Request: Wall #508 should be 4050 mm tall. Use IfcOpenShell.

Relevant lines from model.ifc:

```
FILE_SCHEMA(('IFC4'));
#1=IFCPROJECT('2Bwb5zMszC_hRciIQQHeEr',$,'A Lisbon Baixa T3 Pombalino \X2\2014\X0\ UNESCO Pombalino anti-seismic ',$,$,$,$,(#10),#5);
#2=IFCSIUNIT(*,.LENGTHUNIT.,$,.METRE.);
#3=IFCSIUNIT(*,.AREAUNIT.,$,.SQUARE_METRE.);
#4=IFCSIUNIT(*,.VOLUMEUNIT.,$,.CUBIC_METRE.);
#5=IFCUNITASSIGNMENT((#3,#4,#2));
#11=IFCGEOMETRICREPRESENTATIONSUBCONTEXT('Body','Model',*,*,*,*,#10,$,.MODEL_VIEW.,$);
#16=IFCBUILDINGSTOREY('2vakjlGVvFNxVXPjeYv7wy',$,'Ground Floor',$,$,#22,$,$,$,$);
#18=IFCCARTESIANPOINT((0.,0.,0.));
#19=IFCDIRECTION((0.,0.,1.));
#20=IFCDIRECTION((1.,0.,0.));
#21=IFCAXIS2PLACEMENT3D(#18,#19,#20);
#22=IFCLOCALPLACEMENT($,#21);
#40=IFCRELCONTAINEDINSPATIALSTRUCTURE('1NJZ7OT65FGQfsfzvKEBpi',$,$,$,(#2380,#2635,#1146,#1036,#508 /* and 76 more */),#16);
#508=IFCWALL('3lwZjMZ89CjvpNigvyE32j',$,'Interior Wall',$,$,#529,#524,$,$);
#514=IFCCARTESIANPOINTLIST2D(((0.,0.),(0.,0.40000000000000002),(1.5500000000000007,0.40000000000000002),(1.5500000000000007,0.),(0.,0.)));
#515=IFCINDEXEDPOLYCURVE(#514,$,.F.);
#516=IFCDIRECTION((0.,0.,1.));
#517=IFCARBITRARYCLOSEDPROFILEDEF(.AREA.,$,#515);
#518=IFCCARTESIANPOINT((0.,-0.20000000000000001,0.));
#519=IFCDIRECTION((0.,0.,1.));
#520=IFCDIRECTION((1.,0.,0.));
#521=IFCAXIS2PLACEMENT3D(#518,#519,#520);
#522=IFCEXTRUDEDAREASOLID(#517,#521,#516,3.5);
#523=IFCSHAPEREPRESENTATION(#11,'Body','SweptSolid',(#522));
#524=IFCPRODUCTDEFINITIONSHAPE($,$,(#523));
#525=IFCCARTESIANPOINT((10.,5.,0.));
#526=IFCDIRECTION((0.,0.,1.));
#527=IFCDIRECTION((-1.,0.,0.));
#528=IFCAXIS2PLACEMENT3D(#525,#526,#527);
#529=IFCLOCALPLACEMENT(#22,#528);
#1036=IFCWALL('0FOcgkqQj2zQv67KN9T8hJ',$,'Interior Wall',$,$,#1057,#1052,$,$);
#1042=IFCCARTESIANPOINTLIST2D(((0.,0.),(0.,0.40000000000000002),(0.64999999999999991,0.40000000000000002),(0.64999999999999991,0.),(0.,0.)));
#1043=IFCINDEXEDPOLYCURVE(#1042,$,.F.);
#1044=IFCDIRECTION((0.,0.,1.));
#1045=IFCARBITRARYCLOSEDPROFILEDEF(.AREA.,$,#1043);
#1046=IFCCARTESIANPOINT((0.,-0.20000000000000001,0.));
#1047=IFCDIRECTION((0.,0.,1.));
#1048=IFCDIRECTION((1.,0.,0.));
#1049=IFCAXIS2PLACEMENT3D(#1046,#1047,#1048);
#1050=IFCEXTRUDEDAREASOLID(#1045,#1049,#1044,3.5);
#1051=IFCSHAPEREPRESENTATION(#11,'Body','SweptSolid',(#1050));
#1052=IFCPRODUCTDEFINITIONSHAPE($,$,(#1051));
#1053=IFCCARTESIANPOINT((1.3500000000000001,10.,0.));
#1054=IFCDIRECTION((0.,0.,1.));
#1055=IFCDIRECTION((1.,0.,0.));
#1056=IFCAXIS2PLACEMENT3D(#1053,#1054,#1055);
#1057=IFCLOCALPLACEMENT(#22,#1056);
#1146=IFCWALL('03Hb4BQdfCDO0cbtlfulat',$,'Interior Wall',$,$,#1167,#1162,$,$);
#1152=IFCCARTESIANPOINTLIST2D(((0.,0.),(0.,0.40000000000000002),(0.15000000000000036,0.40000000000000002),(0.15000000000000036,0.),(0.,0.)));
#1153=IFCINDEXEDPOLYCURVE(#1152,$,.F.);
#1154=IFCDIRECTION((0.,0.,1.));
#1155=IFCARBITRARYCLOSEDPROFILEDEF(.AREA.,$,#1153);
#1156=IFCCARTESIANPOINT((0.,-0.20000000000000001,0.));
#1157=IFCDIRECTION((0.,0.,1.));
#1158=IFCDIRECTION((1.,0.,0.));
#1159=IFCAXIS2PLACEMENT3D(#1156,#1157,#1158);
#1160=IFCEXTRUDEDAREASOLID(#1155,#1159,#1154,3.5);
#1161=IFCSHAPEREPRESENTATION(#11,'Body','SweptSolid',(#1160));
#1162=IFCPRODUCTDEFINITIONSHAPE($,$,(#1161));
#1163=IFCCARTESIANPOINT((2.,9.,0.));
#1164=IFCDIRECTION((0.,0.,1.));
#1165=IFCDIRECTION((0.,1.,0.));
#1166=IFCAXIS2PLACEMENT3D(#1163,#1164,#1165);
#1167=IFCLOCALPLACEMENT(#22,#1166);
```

```python
import ifcopenshell
import ifcopenshell.geom
import ifcopenshell.util.representation
import ifcopenshell.util.shape
import ifcopenshell.util.unit

model = ifcopenshell.open("model.ifc")
unit_scale = ifcopenshell.util.unit.calculate_unit_scale(model)
settings = ifcopenshell.geom.settings()


def volume(element):
    """Net volume in cubic metres, openings subtracted."""
    shape = ifcopenshell.geom.create_shape(settings, element)
    return ifcopenshell.util.shape.get_volume(shape.geometry)


wall = model.by_guid("3lwZjMZ89CjvpNigvyE32j")
before = volume(wall)

body = ifcopenshell.util.representation.get_representation(wall, "Model", "Body")
solid = body.Items[0]
old_height = solid.Depth
solid.Depth = 4.05 / unit_scale
after = volume(wall)

print(f"height {old_height:g} -> {solid.Depth:g}, volume {before:.3f} -> {after:.3f} m3")

model.write("model_rev.ifc")
```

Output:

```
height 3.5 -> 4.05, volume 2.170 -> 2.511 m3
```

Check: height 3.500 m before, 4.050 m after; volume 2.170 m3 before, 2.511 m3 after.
